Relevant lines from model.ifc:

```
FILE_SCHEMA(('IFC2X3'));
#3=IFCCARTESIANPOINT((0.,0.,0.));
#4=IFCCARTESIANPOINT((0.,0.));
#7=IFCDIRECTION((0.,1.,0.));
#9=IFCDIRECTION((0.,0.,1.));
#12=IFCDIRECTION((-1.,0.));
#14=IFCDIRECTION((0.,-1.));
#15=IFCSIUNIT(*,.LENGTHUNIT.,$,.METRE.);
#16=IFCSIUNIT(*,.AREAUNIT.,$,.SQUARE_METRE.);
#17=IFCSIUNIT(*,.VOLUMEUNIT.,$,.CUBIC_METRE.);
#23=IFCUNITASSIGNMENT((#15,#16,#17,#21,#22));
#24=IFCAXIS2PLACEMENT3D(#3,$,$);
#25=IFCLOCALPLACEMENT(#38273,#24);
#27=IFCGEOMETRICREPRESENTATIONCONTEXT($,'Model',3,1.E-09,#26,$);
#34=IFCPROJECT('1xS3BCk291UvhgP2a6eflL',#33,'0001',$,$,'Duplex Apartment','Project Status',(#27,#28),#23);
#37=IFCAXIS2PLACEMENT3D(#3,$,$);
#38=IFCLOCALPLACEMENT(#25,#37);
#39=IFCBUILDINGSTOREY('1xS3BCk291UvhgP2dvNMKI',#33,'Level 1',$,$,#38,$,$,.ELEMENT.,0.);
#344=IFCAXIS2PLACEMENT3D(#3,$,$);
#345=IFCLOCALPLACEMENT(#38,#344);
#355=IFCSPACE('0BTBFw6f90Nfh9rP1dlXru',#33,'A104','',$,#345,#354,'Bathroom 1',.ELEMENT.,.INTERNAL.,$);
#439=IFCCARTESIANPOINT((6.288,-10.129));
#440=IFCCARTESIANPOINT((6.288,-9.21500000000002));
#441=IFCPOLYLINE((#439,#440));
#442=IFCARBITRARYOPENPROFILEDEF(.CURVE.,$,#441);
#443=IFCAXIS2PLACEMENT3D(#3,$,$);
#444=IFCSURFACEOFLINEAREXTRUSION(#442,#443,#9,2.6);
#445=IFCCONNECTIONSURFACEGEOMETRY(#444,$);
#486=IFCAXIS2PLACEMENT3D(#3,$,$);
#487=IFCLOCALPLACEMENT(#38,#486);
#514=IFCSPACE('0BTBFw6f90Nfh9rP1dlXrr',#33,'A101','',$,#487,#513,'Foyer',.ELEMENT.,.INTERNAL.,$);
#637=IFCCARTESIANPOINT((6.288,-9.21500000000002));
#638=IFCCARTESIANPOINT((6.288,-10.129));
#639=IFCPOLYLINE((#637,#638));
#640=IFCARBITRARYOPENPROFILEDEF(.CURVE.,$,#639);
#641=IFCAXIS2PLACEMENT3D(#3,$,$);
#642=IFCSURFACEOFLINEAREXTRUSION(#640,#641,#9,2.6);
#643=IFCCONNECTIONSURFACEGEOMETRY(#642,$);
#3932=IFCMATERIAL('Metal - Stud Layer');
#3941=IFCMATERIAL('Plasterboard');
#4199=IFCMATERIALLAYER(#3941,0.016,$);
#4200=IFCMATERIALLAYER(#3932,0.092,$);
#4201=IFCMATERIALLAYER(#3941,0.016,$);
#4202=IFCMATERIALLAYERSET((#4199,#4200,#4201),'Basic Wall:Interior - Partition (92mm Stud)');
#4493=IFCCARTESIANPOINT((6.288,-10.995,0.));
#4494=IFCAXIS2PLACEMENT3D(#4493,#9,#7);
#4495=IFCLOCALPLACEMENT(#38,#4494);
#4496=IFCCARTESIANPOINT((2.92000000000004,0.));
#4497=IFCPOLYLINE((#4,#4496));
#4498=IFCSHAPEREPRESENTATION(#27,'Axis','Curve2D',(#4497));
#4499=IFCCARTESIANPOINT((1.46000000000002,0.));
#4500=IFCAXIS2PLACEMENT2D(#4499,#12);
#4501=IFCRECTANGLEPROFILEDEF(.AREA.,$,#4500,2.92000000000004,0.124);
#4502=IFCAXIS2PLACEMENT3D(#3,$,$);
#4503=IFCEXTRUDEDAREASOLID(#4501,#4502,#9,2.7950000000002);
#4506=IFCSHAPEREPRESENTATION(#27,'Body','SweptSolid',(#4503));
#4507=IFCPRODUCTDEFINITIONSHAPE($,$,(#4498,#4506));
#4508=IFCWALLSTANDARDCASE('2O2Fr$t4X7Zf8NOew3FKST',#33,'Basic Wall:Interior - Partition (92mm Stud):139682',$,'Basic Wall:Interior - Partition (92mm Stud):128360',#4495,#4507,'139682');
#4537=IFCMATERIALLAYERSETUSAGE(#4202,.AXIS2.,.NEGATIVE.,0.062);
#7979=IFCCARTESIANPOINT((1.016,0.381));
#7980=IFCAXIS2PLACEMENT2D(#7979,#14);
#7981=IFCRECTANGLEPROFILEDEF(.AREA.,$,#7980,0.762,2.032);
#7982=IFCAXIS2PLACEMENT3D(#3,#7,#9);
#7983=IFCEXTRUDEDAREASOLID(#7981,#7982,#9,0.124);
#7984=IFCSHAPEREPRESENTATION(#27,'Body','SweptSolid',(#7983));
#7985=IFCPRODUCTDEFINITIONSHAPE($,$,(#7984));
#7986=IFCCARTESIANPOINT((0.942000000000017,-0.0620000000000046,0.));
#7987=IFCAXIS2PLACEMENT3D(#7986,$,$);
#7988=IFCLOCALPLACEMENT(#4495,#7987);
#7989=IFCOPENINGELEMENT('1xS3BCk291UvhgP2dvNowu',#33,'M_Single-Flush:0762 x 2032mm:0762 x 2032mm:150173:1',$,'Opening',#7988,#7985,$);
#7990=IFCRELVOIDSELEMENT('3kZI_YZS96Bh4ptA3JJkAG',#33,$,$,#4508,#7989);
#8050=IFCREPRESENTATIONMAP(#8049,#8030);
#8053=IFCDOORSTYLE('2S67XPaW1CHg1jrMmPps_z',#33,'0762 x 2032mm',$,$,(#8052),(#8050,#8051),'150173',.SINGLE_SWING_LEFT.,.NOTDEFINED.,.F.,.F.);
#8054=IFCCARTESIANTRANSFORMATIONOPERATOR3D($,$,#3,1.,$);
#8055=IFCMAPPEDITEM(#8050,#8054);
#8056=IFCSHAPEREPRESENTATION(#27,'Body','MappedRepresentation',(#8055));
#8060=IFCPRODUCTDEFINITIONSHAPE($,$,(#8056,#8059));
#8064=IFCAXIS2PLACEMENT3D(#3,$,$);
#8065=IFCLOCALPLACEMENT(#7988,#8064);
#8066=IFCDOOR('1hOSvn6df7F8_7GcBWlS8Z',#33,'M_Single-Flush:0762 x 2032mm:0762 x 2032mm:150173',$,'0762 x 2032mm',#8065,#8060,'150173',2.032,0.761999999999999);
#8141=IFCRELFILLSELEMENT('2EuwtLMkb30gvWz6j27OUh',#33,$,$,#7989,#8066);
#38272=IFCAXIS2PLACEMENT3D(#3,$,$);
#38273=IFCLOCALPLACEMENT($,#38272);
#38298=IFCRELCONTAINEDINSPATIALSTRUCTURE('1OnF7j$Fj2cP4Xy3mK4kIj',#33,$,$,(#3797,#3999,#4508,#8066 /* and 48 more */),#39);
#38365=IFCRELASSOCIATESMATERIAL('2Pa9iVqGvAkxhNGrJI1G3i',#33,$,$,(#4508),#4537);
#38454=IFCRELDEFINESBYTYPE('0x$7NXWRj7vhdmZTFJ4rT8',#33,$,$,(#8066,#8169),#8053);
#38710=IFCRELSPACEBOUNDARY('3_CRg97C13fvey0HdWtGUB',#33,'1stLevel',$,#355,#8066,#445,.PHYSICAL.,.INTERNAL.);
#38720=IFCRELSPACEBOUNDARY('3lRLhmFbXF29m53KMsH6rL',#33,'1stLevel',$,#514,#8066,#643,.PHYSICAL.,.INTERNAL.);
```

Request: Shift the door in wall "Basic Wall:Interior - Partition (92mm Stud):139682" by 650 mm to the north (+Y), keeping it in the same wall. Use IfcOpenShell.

```python
import numpy as np
import ifcopenshell
import ifcopenshell.api.geometry
import ifcopenshell.util.placement

model = ifcopenshell.open("model.ifc")

door = model.by_id(8066)
opening = door.FillsVoids[0].RelatingOpeningElement
wall = opening.VoidsElements[0].RelatingBuildingElement

wall_matrix = ifcopenshell.util.placement.get_local_placement(wall.ObjectPlacement)
shift = wall_matrix[:3, 0] * 0.65
before = ifcopenshell.util.placement.get_local_placement(door.ObjectPlacement)[:3, 3].copy()

# The door is placed relative to its opening, so it follows when the opening moves.
matrix = ifcopenshell.util.placement.get_local_placement(opening.ObjectPlacement)
matrix[:3, 3] += shift
ifcopenshell.api.geometry.edit_object_placement(
    model, product=opening, matrix=matrix, is_si=False, should_transform_children=True
)

# Space boundary surfaces are stored in each space's coordinates; move them too.
for rel in door.ProvidesBoundaries:
    if not rel.ConnectionGeometry:
        continue
    surface = rel.ConnectionGeometry.SurfaceOnRelatingElement
    space_matrix = ifcopenshell.util.placement.get_local_placement(rel.RelatingSpace.ObjectPlacement)
    point = np.array(surface.Position.Location.Coordinates) + space_matrix[:3, :3].T @ shift
    surface.Position = model.createIfcAxis2Placement3D(
        model.createIfcCartesianPoint(point.tolist()), surface.Position.Axis, surface.Position.RefDirection
    )

after = ifcopenshell.util.placement.get_local_placement(door.ObjectPlacement)[:3, 3]
print("door moved by", (after - before).round(3) + 0.0)

model.write("model_v2.ifc")
```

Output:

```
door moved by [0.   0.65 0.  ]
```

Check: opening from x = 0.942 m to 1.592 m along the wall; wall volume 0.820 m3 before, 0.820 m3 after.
